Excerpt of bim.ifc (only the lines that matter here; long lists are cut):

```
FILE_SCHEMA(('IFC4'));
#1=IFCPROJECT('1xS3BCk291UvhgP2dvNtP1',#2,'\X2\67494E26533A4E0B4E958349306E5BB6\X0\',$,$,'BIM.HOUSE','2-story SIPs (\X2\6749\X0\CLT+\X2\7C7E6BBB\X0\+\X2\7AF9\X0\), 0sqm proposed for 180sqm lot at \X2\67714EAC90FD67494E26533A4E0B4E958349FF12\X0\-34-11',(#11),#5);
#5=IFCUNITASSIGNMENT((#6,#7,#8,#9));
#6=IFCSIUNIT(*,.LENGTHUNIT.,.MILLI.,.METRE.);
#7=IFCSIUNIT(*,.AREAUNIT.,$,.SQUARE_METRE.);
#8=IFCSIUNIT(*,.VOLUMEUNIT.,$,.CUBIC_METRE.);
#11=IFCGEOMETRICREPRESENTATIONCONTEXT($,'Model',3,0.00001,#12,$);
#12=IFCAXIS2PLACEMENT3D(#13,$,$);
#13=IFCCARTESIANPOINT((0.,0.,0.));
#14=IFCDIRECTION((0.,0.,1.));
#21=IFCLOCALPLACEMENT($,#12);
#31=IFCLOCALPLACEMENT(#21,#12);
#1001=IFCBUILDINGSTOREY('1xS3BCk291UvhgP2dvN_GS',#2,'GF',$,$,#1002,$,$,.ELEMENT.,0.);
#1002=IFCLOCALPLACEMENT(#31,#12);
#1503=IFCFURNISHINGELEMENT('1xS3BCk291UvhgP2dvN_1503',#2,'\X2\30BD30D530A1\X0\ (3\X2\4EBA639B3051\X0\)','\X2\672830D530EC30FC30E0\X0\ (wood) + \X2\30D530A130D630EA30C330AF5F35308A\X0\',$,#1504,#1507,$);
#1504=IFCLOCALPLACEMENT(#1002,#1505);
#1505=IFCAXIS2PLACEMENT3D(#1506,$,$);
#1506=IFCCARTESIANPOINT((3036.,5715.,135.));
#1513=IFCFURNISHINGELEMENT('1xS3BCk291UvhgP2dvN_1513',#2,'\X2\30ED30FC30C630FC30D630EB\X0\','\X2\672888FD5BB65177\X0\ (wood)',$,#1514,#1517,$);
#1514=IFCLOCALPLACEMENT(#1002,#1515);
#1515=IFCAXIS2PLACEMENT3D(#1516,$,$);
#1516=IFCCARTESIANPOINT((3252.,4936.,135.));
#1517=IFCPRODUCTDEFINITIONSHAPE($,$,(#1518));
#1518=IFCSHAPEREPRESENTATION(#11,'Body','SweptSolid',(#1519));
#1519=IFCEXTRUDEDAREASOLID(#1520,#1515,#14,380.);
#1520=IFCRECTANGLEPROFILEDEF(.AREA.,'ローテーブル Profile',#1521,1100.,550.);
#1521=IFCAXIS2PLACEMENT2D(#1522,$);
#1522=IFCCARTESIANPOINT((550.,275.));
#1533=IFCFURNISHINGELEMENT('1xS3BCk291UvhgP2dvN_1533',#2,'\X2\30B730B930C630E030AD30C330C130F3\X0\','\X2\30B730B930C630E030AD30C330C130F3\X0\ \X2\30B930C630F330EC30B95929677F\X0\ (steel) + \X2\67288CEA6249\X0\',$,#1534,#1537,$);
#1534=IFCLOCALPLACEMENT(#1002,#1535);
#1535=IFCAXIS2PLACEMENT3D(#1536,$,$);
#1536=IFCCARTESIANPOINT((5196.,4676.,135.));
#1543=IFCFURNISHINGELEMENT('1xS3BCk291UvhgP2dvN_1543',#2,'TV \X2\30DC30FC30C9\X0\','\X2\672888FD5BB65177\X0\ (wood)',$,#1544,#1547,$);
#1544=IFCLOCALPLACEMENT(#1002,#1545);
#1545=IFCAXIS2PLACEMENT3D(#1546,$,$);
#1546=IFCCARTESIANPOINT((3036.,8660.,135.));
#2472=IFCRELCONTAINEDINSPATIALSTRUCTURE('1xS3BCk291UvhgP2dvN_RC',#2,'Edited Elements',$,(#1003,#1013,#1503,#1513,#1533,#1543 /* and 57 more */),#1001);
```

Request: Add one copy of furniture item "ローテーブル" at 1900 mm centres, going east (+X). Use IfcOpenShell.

```python
import numpy as np
import ifcopenshell
import ifcopenshell.api.geometry
import ifcopenshell.api.root
import ifcopenshell.util.element
import ifcopenshell.util.placement

model = ifcopenshell.open("bim.ifc")


def reuse_history(source, copy):
    """copy_class also copies each property set's owner history, people and application; keep the originals."""
    for rel in copy.IsDefinedBy:
        if rel.is_a("IfcRelDefinesByProperties") and (history := rel.RelatingPropertyDefinition.OwnerHistory):
            rel.RelatingPropertyDefinition.OwnerHistory = source.OwnerHistory
            ifcopenshell.util.element.remove_deep2(model, history)


source = model.by_guid("1xS3BCk291UvhgP2dvN_1513")
base = ifcopenshell.util.placement.get_local_placement(source.ObjectPlacement)
step = np.array([1.0, 0.0, 0.0]) * 1900.0

for i in range(1, 2):
    copy = ifcopenshell.api.root.copy_class(model, product=source)
    copy.Representation = ifcopenshell.util.element.copy_deep(
        model, source.Representation, exclude=["IfcGeometricRepresentationContext", "IfcRepresentationMap"]
    )
    reuse_history(source, copy)
    matrix = base.copy()
    matrix[:3, 3] += i * step
    print("added at", matrix[:3, 3].round(3) + 0.0)
    ifcopenshell.api.geometry.edit_object_placement(model, product=copy, matrix=matrix, is_si=False)

model.write("bim_edited.ifc")
```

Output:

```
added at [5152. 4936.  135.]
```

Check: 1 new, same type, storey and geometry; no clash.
